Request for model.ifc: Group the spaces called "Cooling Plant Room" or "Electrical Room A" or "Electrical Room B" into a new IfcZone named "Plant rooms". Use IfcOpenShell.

First a look at what the model holds.

```python
import ifcopenshell

model = ifcopenshell.open("model.ifc")
print(model.schema)
seen = {}
for space in model.by_type("IfcSpace"):
    seen[space.LongName] = seen.get(space.LongName, 0) + 1
for name, count in sorted(seen.items(), key=str):
    print(count, "x", name)
print("zones:", [z.Name for z in model.by_type("IfcZone")][:20])
```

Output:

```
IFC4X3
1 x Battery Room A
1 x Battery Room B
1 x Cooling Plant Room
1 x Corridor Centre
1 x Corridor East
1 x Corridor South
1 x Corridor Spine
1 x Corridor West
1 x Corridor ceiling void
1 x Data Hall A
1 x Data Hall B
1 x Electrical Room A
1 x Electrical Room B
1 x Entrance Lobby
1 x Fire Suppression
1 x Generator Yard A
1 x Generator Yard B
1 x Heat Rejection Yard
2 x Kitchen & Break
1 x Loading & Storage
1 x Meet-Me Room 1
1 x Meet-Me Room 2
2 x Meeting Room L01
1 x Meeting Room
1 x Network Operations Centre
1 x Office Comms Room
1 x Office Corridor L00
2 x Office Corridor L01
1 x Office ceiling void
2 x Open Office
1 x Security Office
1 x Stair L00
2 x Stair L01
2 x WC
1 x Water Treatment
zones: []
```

```python
import ifcopenshell
import ifcopenshell.api.group
import ifcopenshell.api.root

model = ifcopenshell.open("model.ifc")

names = {"Cooling Plant Room", "Electrical Room A", "Electrical Room B"}
spaces = [s for s in model.by_type("IfcSpace") if s.LongName in names]

zone = ifcopenshell.api.root.create_entity(model, ifc_class="IfcZone", name="Plant rooms")
ifcopenshell.api.group.assign_group(model, products=spaces, group=zone)
print(len(spaces), "spaces in", zone.Name)

model.write("model_edited.ifc")
```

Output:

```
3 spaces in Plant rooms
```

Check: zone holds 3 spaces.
